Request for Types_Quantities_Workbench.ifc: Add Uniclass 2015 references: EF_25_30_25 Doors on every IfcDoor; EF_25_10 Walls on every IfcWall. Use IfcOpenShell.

First a look at what the model holds.

```python
import ifcopenshell

model = ifcopenshell.open("Types_Quantities_Workbench.ifc")
print(model.schema)
print("classifications:", [c.Name for c in model.by_type("IfcClassification")])
for ifc_class in ("IfcDoor", "IfcRoof", "IfcStair", "IfcWall", "IfcWindow"):
    print(ifc_class, len(model.by_type(ifc_class)))
```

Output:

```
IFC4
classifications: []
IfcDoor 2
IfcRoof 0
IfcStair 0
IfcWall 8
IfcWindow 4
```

```python
import ifcopenshell
import ifcopenshell.api.classification

model = ifcopenshell.open("Types_Quantities_Workbench.ifc")

system = ifcopenshell.api.classification.add_classification(model, classification="Uniclass 2015")

codes = {
    "IfcDoor": ("EF_25_30_25", "Doors"),
    "IfcWall": ("EF_25_10", "Walls"),
}
for ifc_class, (code, name) in codes.items():
    products = model.by_type(ifc_class)
    ifcopenshell.api.classification.add_reference(
        model, products=products, classification=system, identification=code, name=name
    )
    print(code, len(products))

model.write("Types_Quantities_Workbench_edited.ifc")
```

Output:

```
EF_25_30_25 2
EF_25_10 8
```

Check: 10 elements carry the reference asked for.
